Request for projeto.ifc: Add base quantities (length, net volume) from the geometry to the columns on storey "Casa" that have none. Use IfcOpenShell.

First a look at what the model holds.

```python
import ifcopenshell
import ifcopenshell.util.element
import ifcopenshell.util.unit

model = ifcopenshell.open("projeto.ifc")
print(model.schema)
for unit_type in ("LENGTHUNIT", "AREAUNIT", "VOLUMEUNIT"):
    print(unit_type, ifcopenshell.util.unit.calculate_unit_scale(model, unit_type))
storey = next(s for s in model.by_type("IfcBuildingStorey") if s.Name == "Casa")
columns = [e for e in ifcopenshell.util.element.get_decomposition(storey) if e.is_a("IfcColumn")]
for e in sorted(columns, key=lambda e: e.id()):
    print(e.id(), e.is_a(), e.Name, list(ifcopenshell.util.element.get_psets(e, qtos_only=True)), sep=" | ")
```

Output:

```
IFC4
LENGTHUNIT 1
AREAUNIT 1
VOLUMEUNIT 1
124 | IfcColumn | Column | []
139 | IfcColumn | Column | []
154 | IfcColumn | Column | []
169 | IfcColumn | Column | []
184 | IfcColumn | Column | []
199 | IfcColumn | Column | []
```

```python
import ifcopenshell
import ifcopenshell.api.pset
import ifcopenshell.geom
import ifcopenshell.util.element
import ifcopenshell.util.shape
import ifcopenshell.util.unit

model = ifcopenshell.open("projeto.ifc")
unit_scale = ifcopenshell.util.unit.calculate_unit_scale(model)
volume_scale = ifcopenshell.util.unit.calculate_unit_scale(model, "VOLUMEUNIT")
settings = ifcopenshell.geom.settings()

storey = next(s for s in model.by_type("IfcBuildingStorey") if s.Name == "Casa")
columns = [e for e in ifcopenshell.util.element.get_decomposition(storey) if e.is_a("IfcColumn")]

for e in sorted(columns, key=lambda e: e.id()):
    if ifcopenshell.util.element.get_psets(e, qtos_only=True, should_inherit=False):
        continue
    # Geometry comes back in metres, in the element's own axes.
    shape = ifcopenshell.geom.create_shape(settings, e)
    values = {
        "Length": ifcopenshell.util.shape.get_z(shape.geometry) / unit_scale,
        "NetVolume": ifcopenshell.util.shape.get_volume(shape.geometry) / volume_scale,
    }
    qto = ifcopenshell.api.pset.add_qto(model, product=e, name="Qto_ColumnBaseQuantities")
    ifcopenshell.api.pset.edit_qto(model, qto=qto, properties=values)
    print(e.id(), {k: round(v, 3) for k, v in values.items()})

model.write("projeto_updated.ifc")
```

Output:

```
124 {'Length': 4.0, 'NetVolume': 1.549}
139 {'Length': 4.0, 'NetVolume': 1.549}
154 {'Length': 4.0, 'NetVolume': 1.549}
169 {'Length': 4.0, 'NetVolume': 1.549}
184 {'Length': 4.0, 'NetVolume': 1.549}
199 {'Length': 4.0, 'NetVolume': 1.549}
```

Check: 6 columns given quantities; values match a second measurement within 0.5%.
